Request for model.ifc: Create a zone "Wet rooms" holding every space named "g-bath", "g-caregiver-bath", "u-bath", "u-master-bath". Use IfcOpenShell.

First a look at what the model holds.

```python
import ifcopenshell

model = ifcopenshell.open("model.ifc")
print(model.schema)
seen = {}
for space in model.by_type("IfcSpace"):
    seen[space.LongName] = seen.get(space.LongName, 0) + 1
for name, count in sorted(seen.items(), key=str):
    print(count, "x", name)
print("zones:", [z.Name for z in model.by_type("IfcZone")][:20])
```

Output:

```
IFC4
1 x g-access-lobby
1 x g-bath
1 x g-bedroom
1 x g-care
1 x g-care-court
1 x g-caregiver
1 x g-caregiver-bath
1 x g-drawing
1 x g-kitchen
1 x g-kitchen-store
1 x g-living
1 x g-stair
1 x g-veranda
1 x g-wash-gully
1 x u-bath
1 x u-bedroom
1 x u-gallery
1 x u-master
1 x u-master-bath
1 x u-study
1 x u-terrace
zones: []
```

```python
import ifcopenshell
import ifcopenshell.api.group
import ifcopenshell.api.root

model = ifcopenshell.open("model.ifc")

names = {"g-bath", "g-caregiver-bath", "u-bath", "u-master-bath"}
spaces = [s for s in model.by_type("IfcSpace") if s.LongName in names]

zone = ifcopenshell.api.root.create_entity(model, ifc_class="IfcZone", name="Wet rooms")
ifcopenshell.api.group.assign_group(model, products=spaces, group=zone)
print(len(spaces), "spaces in", zone.Name)

model.write("model-out.ifc")
```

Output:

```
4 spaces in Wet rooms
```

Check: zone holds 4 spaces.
